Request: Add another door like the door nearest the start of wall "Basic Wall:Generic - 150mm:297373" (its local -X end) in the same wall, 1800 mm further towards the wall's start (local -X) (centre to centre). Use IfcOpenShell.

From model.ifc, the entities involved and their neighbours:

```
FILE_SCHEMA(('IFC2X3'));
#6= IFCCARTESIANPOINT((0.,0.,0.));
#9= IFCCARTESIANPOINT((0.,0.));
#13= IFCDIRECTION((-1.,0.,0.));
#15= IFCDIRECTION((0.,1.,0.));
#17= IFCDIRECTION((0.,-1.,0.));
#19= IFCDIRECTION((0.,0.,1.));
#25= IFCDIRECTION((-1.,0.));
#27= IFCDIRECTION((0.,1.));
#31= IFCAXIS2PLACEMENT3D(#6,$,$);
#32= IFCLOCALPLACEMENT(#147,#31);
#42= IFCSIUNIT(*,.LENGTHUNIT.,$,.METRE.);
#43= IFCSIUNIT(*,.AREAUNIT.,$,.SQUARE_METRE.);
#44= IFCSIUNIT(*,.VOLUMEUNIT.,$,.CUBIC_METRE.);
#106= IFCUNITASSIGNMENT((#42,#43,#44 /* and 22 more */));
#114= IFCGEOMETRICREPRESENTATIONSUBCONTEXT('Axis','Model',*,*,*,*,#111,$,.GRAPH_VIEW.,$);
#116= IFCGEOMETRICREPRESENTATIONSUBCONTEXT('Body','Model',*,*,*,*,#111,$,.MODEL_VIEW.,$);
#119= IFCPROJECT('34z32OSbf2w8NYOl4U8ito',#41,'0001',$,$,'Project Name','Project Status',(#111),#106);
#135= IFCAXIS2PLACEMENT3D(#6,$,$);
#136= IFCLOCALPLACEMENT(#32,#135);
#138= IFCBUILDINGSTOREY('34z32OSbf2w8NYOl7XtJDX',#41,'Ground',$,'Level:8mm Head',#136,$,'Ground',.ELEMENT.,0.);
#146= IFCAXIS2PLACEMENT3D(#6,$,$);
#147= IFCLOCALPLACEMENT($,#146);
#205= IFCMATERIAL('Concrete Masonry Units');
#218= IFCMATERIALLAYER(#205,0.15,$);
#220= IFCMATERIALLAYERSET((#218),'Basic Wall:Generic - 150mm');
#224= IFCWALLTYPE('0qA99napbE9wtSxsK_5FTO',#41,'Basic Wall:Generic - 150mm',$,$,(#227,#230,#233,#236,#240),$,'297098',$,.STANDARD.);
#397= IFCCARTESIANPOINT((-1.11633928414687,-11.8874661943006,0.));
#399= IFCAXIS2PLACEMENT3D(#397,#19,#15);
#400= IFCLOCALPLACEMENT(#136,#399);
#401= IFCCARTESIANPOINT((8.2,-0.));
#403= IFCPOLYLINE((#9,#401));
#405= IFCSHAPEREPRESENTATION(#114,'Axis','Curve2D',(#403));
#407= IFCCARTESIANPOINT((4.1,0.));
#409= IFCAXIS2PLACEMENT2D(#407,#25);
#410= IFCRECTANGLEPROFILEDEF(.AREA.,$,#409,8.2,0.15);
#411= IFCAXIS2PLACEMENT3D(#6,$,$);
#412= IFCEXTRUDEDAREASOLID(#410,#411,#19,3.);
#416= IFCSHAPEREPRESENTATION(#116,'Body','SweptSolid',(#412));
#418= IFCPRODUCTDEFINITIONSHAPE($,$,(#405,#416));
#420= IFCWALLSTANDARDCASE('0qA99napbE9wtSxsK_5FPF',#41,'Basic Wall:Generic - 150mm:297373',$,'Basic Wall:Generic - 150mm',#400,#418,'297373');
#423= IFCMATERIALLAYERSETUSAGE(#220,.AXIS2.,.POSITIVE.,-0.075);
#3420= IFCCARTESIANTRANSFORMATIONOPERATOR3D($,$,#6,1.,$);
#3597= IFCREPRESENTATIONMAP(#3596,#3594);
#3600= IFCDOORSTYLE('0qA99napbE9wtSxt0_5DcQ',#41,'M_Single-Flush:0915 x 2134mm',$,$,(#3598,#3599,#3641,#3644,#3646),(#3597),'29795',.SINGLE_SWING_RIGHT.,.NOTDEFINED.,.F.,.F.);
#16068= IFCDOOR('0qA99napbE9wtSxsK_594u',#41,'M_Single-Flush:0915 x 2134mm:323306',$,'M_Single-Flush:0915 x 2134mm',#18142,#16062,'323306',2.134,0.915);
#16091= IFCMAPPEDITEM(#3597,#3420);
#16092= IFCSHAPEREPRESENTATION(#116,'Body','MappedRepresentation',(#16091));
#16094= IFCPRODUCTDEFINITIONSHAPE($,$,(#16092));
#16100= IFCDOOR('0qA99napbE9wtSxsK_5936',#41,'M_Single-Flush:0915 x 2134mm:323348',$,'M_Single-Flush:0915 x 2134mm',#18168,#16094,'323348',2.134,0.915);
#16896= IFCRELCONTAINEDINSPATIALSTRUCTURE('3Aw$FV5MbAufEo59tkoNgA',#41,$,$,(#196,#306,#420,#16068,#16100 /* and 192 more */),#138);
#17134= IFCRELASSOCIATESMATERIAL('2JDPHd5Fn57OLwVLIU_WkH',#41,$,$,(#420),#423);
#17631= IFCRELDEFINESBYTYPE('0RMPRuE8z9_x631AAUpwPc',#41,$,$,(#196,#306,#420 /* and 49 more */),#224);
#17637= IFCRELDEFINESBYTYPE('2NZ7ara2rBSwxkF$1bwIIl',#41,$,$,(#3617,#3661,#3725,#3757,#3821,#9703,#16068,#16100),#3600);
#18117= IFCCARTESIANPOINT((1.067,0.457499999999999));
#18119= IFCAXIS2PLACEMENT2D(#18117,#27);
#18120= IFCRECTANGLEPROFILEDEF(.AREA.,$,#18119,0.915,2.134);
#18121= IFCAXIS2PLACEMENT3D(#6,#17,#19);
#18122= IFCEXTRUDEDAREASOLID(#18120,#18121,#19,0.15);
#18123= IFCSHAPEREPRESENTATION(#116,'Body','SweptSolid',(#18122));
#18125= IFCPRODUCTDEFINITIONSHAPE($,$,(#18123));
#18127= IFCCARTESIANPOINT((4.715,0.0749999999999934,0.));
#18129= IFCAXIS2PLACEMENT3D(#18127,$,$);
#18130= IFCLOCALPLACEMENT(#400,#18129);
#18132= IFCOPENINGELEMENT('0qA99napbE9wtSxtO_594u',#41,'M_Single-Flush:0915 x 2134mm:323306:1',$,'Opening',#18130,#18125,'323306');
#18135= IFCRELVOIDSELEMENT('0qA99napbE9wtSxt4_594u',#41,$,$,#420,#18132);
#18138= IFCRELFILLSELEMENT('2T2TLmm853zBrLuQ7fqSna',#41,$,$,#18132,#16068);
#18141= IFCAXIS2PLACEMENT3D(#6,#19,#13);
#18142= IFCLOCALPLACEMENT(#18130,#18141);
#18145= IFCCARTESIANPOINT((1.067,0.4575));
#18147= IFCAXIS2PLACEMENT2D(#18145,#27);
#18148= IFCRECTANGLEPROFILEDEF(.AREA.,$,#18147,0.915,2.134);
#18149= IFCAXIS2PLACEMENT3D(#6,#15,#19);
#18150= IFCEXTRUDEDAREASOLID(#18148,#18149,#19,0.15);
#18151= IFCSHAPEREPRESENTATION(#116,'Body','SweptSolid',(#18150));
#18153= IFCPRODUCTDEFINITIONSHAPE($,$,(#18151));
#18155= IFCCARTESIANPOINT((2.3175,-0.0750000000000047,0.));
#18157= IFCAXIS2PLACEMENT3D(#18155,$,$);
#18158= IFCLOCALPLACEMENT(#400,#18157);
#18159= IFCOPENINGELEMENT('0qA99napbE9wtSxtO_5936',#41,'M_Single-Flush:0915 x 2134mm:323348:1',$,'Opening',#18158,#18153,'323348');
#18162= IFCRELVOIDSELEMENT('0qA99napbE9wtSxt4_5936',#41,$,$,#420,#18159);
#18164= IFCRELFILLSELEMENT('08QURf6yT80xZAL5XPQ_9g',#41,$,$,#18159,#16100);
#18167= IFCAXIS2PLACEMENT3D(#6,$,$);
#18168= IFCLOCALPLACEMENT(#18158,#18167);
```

```python
import ifcopenshell
import ifcopenshell.api.feature
import ifcopenshell.api.geometry
import ifcopenshell.api.root
import ifcopenshell.geom
import ifcopenshell.util.element
import ifcopenshell.util.placement
import ifcopenshell.util.shape
import ifcopenshell.util.unit

model = ifcopenshell.open("model.ifc")
unit_scale = ifcopenshell.util.unit.calculate_unit_scale(model)
settings = ifcopenshell.geom.settings()


def volume(element):
    """Net volume in cubic metres, openings subtracted."""
    shape = ifcopenshell.geom.create_shape(settings, element)
    return ifcopenshell.util.shape.get_volume(shape.geometry)


def reuse_history(source, copy):
    """copy_class also copies each property set's owner history, people and application; keep the originals."""
    for rel in copy.IsDefinedBy:
        if rel.is_a("IfcRelDefinesByProperties") and (history := rel.RelatingPropertyDefinition.OwnerHistory):
            rel.RelatingPropertyDefinition.OwnerHistory = source.OwnerHistory
            ifcopenshell.util.element.remove_deep2(model, history)


door = model.by_id(16100)
opening = door.FillsVoids[0].RelatingOpeningElement
wall = opening.VoidsElements[0].RelatingBuildingElement
before = volume(wall)
shift = ifcopenshell.util.placement.get_local_placement(wall.ObjectPlacement)[:3, 0] * -1.8 / unit_scale

# copy_class copies the void relationship, type, container and properties, but no geometry.
new_opening = ifcopenshell.api.root.copy_class(model, product=opening)
new_opening.Representation = ifcopenshell.util.element.copy_deep(
    model, opening.Representation, exclude=["IfcGeometricRepresentationContext", "IfcRepresentationMap"]
)
new_opening.Name = "M_Single-Flush:0915 x 2134mm"
new_opening.Tag = None
new_door = ifcopenshell.api.root.copy_class(model, product=door)
new_door.Representation = ifcopenshell.util.element.copy_deep(
    model, door.Representation, exclude=["IfcGeometricRepresentationContext", "IfcRepresentationMap"]
)
new_door.Name = "M_Single-Flush:0915 x 2134mm"
new_door.Tag = None
reuse_history(door, new_door)
fills = ifcopenshell.api.feature.add_filling(model, opening=new_opening, element=new_door)
fills.OwnerHistory = new_door.OwnerHistory  # required in IFC2X3

for old, new in ((opening, new_opening), (door, new_door)):
    matrix = ifcopenshell.util.placement.get_local_placement(old.ObjectPlacement)
    matrix[:3, 3] += shift
    ifcopenshell.api.geometry.edit_object_placement(model, product=new, matrix=matrix, is_si=False)

after = volume(wall)

print(f"wall volume {before:.3f} -> {after:.3f} m3")

model.write("model_rev.ifc")
```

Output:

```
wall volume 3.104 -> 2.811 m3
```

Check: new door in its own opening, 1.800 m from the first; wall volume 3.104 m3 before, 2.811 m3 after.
